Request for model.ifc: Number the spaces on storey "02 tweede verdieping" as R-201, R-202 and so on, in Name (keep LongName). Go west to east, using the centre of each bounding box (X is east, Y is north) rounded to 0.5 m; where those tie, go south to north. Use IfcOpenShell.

First a look at what the model holds.

```python
import ifcopenshell
import ifcopenshell.util.element
import ifcopenshell.util.placement

model = ifcopenshell.open("model.ifc")
print(model.schema)
storey = next(s for s in model.by_type("IfcBuildingStorey") if s.Name == "02 tweede verdieping")
spaces = [e for e in ifcopenshell.util.element.get_decomposition(storey) if e.is_a("IfcSpace")]
for e in sorted(spaces, key=lambda e: e.id()):
    origin = ifcopenshell.util.placement.get_local_placement(e.ObjectPlacement)[:3, 3]
    print(e.id(), e.Name, e.LongName, origin.round(2) + 0.0, sep=" | ")
```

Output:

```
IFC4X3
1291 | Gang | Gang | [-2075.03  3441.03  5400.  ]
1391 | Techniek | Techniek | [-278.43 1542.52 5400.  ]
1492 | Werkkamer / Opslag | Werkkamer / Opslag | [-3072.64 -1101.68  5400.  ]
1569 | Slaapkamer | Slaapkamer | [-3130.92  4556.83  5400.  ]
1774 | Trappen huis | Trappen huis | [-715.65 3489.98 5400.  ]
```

```python
import ifcopenshell
import ifcopenshell.geom
import ifcopenshell.util.element
import ifcopenshell.util.shape

model = ifcopenshell.open("model.ifc")
settings = ifcopenshell.geom.settings()
settings.set("use-world-coords", True)


def centre(element):
    shape = ifcopenshell.geom.create_shape(settings, element)
    return ifcopenshell.util.shape.get_bbox_centroid(shape.geometry)


storey = next(s for s in model.by_type("IfcBuildingStorey") if s.Name == "02 tweede verdieping")
spaces = [e for e in ifcopenshell.util.element.get_decomposition(storey) if e.is_a("IfcSpace")]

# Insertion points can sit at a corner or the storey origin, so sort by the geometry (in metres).
centres = {e: centre(e) for e in spaces}
spaces.sort(key=lambda e: (round(centres[e][0] / 0.5), centres[e][1]))

for i, e in enumerate(spaces, start=1):
    number = f"R-2{i:02d}"
    e.Name = number
    print(e.id(), number)

model.write("model_updated.ifc")
```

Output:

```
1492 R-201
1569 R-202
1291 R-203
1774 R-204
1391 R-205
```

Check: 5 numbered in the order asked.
